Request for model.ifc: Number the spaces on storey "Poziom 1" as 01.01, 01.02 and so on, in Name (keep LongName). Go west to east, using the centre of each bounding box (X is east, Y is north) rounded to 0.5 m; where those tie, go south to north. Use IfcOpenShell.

First a look at what the model holds.

```python
import ifcopenshell
import ifcopenshell.util.element
import ifcopenshell.util.placement

model = ifcopenshell.open("model.ifc")
print(model.schema)
storey = next(s for s in model.by_type("IfcBuildingStorey") if s.Name == "Poziom 1")
spaces = [e for e in ifcopenshell.util.element.get_decomposition(storey) if e.is_a("IfcSpace")]
for e in sorted(spaces, key=lambda e: e.id()):
    origin = ifcopenshell.util.placement.get_local_placement(e.ObjectPlacement)[:3, 3]
    print(e.id(), e.Name, e.LongName, origin.round(2) + 0.0, sep=" | ")
```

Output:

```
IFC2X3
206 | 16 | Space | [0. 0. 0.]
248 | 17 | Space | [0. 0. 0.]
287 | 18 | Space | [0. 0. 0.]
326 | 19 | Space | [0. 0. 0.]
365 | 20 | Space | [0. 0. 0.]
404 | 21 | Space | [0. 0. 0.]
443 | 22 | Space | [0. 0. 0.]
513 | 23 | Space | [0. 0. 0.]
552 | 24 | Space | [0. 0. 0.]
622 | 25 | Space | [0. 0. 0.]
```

```python
import ifcopenshell
import ifcopenshell.geom
import ifcopenshell.util.element
import ifcopenshell.util.shape

model = ifcopenshell.open("model.ifc")
settings = ifcopenshell.geom.settings()
settings.set("use-world-coords", True)


def centre(element):
    shape = ifcopenshell.geom.create_shape(settings, element)
    return ifcopenshell.util.shape.get_bbox_centroid(shape.geometry)


storey = next(s for s in model.by_type("IfcBuildingStorey") if s.Name == "Poziom 1")
spaces = [e for e in ifcopenshell.util.element.get_decomposition(storey) if e.is_a("IfcSpace")]

# Insertion points can sit at a corner or the storey origin, so sort by the geometry (in metres).
centres = {e: centre(e) for e in spaces}
spaces.sort(key=lambda e: (round(centres[e][0] / 0.5), centres[e][1]))

for i, e in enumerate(spaces, start=1):
    number = f"01.{i:02d}"
    e.Name = number
    print(e.id(), number)

model.write("model_updated.ifc")
```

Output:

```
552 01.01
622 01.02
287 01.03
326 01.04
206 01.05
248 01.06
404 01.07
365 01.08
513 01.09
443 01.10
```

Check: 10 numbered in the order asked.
